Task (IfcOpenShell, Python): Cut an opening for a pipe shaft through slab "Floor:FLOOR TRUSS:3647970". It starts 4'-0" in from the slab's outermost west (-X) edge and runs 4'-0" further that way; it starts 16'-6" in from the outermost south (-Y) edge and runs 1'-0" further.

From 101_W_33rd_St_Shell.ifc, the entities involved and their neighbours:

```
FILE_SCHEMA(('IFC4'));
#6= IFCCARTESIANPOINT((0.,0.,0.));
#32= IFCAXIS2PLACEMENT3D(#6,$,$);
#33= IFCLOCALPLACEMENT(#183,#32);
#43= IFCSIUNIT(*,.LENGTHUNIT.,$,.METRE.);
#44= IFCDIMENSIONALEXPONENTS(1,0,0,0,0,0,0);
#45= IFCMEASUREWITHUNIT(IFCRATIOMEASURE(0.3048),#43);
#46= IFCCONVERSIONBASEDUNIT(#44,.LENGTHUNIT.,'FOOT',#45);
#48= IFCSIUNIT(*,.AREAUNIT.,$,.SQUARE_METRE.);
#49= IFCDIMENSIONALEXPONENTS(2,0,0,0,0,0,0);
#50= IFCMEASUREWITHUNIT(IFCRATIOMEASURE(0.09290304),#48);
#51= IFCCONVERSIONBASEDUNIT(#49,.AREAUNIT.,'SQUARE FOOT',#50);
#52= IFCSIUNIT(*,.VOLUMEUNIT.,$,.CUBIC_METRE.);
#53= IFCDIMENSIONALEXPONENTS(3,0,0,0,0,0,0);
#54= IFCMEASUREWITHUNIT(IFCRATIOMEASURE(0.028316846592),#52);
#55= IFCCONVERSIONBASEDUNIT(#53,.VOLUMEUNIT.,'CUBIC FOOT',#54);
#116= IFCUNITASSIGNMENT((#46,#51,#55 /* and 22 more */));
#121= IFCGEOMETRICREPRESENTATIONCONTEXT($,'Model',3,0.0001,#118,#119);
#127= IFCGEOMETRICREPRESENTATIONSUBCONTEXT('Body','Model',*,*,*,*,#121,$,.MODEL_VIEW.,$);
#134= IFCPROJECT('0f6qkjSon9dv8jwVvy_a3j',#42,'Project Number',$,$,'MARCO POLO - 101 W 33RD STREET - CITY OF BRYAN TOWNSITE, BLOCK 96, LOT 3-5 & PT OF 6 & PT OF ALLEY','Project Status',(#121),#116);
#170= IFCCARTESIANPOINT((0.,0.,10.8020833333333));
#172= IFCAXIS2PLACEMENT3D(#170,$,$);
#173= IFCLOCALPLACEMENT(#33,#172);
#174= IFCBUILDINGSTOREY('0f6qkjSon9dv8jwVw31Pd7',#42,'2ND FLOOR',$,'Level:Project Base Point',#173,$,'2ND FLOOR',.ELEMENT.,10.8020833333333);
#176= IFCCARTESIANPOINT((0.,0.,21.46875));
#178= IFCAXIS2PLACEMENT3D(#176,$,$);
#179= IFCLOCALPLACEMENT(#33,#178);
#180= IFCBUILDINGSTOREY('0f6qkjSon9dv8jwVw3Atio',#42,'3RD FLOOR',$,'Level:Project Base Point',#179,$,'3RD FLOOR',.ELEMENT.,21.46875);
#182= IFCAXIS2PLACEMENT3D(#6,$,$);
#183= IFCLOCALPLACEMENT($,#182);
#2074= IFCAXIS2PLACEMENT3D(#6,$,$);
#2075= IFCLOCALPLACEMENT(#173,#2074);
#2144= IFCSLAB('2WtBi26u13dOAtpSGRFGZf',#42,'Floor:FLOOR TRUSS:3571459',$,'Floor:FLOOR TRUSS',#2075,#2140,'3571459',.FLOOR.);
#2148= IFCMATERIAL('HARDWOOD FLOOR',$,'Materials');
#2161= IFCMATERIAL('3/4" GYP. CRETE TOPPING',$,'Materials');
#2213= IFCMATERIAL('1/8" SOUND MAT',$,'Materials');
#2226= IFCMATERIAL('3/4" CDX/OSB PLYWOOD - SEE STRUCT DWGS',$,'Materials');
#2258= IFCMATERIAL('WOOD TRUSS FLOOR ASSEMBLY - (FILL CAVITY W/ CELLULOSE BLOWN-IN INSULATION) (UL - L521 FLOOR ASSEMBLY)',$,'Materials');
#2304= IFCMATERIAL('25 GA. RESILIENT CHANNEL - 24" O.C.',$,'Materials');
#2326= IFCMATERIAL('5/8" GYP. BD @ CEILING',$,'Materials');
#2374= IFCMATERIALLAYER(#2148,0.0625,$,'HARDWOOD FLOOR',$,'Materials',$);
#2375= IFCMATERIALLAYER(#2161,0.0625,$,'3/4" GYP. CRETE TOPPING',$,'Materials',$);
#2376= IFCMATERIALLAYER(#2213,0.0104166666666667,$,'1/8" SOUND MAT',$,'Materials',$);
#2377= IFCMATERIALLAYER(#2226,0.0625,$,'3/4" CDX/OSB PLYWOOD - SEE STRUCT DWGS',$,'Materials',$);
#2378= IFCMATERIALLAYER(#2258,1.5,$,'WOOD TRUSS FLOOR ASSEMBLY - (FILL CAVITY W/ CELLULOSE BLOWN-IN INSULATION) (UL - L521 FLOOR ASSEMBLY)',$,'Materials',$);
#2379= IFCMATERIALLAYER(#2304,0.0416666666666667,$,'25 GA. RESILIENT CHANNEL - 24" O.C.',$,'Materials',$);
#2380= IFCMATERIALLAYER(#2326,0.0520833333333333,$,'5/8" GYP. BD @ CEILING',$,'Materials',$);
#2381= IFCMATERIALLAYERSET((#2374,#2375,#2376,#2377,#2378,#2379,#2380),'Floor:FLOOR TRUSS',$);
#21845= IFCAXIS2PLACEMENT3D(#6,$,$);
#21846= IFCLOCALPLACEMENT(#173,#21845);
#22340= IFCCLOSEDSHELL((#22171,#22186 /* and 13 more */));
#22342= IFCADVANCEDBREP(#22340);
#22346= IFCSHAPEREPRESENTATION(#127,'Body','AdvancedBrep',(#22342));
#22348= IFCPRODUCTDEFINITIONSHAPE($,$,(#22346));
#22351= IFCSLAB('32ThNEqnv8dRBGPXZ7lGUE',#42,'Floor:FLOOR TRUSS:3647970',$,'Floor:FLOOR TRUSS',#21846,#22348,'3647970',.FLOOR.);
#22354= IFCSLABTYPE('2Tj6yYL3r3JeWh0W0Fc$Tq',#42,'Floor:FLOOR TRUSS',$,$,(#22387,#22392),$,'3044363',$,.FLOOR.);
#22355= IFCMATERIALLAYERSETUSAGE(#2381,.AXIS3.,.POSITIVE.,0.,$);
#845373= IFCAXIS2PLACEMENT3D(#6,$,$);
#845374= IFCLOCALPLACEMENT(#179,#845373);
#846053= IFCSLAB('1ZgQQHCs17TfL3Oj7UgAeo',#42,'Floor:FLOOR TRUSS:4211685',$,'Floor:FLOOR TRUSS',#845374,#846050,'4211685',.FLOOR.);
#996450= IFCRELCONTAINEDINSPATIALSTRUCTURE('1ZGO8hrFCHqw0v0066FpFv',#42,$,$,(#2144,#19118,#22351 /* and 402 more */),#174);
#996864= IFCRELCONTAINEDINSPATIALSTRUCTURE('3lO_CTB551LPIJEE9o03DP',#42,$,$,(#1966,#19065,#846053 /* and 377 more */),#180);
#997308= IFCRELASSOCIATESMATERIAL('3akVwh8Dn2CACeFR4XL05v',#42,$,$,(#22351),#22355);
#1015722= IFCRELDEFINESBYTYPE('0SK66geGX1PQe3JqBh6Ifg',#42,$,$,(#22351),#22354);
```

```python
import numpy as np
import ifcopenshell
import ifcopenshell.api.feature
import ifcopenshell.api.geometry
import ifcopenshell.api.root
import ifcopenshell.geom
import ifcopenshell.util.placement
import ifcopenshell.util.representation
import ifcopenshell.util.shape
import ifcopenshell.util.unit

model = ifcopenshell.open("101_W_33rd_St_Shell.ifc")
unit_scale = ifcopenshell.util.unit.calculate_unit_scale(model)
settings = ifcopenshell.geom.settings()


def volume(element):
    """Net volume in cubic metres, openings subtracted."""
    shape = ifcopenshell.geom.create_shape(settings, element)
    return ifcopenshell.util.shape.get_volume(shape.geometry)


slab = model.by_id(22351)
before = volume(slab)

# Extent in the slab's own axes, in metres. The edges named are its -X and -Y sides.
slab_shape = ifcopenshell.geom.create_shape(settings, slab)
vertices = ifcopenshell.util.shape.get_vertices(slab_shape.geometry)
x_min, y_min, bottom = vertices.min(axis=0)
top = vertices[:, 2].max()

opening = ifcopenshell.api.root.create_entity(model, ifc_class="IfcOpeningElement", name="Pipe shaft opening", predefined_type="OPENING")
context = ifcopenshell.util.representation.get_context(model, "Model", "Body", "MODEL_VIEW")
width, depth = 1.2192, 0.3048
outline = [(0.0, 0.0), (width, 0.0), (width, depth), (0.0, depth), (0.0, 0.0)]
# Overshoot both faces by 50 mm so the cut is clean.
shape = ifcopenshell.api.geometry.add_slab_representation(
    model, context=context, depth=top - bottom + 0.1, polyline=outline
)
ifcopenshell.api.geometry.assign_representation(model, product=opening, representation=shape)

matrix = ifcopenshell.util.placement.get_local_placement(slab.ObjectPlacement)
matrix[:, 3] = matrix @ np.append(np.array([x_min + 1.2192, y_min + 5.0292, bottom - 0.05]) / unit_scale, 1.0)
ifcopenshell.api.geometry.edit_object_placement(model, product=opening, matrix=matrix, is_si=False)
ifcopenshell.api.feature.add_feature(model, feature=opening, element=slab)

after = volume(slab)

print(f"slab volume {before:.3f} -> {after:.3f} m3")

model.write("101_W_33rd_St_Shell_updated.ifc")
```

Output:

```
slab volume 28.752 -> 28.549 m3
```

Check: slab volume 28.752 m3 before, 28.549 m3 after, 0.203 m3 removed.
